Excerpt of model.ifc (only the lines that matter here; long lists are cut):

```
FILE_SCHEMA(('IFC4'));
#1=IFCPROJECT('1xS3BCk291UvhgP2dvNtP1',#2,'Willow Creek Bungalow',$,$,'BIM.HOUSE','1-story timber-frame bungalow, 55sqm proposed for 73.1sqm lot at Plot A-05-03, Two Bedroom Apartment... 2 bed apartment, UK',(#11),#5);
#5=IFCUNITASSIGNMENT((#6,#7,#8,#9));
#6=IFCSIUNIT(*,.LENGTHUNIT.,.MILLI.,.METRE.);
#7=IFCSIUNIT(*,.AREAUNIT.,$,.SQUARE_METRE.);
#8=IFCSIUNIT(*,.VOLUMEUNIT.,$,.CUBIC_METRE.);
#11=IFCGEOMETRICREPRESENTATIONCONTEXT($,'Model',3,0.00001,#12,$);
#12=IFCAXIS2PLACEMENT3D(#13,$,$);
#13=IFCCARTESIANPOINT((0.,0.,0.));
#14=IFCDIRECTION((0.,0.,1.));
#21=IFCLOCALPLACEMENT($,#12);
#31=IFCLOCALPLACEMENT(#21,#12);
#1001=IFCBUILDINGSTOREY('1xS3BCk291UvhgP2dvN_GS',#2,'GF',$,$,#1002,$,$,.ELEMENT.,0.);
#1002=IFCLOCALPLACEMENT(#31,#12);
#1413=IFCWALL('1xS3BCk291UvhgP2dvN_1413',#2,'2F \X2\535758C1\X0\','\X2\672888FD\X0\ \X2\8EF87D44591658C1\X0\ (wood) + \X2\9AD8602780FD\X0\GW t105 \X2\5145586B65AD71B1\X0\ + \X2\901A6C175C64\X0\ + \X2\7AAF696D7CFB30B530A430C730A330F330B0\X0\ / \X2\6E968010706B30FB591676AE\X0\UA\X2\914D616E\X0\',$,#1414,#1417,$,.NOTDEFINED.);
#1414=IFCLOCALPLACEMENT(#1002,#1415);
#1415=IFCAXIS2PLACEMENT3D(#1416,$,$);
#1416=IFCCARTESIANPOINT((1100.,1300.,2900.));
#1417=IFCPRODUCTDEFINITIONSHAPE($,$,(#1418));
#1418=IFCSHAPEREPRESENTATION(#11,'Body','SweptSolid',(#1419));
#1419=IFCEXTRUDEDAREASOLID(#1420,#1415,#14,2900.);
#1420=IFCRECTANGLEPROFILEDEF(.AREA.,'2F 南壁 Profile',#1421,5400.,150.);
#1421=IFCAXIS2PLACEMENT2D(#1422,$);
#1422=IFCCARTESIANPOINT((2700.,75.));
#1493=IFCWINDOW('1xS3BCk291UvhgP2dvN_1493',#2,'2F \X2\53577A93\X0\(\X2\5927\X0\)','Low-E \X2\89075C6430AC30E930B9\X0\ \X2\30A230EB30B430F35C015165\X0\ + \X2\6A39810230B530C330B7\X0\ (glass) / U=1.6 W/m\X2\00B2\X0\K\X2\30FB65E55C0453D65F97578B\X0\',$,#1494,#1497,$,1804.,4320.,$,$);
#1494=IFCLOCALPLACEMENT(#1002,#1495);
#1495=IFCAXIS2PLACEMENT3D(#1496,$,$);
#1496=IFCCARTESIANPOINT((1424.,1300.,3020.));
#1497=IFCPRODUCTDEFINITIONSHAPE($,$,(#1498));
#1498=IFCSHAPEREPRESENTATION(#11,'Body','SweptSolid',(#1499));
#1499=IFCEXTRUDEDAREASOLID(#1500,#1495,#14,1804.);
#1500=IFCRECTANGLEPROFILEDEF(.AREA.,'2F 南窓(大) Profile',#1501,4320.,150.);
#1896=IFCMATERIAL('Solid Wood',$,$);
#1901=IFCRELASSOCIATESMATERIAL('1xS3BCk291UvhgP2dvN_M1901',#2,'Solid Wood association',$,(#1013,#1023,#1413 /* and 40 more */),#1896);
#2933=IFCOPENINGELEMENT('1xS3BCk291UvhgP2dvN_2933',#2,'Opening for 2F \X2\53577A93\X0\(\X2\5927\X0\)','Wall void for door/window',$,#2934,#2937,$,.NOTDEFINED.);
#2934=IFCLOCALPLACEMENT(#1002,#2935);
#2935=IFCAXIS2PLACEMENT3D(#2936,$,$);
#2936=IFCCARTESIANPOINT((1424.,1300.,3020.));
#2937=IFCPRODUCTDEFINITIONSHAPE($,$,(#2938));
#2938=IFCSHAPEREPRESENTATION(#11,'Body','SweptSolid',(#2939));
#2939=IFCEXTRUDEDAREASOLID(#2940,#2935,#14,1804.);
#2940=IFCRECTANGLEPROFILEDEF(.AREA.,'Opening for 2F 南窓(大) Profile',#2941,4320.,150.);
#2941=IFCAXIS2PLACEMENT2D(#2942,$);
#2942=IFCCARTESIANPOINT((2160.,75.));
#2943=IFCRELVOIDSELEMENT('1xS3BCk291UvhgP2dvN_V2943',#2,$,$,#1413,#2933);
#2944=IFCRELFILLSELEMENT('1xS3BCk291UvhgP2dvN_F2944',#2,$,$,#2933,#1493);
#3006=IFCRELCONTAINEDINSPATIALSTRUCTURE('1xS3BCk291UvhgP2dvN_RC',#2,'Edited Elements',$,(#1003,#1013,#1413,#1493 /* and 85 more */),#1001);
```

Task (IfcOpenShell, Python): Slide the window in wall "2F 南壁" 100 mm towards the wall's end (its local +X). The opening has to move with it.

```python
import ifcopenshell
import ifcopenshell.api.geometry
import ifcopenshell.util.placement
import ifcopenshell.util.unit

model = ifcopenshell.open("model.ifc")
unit_scale = ifcopenshell.util.unit.calculate_unit_scale(model)

window = model.by_guid("1xS3BCk291UvhgP2dvN_1493")
opening = window.FillsVoids[0].RelatingOpeningElement
wall = opening.VoidsElements[0].RelatingBuildingElement

wall_matrix = ifcopenshell.util.placement.get_local_placement(wall.ObjectPlacement)
shift = wall_matrix[:3, 0] * 0.1 / unit_scale
before = ifcopenshell.util.placement.get_local_placement(window.ObjectPlacement)[:3, 3].copy()

# The window is not placed relative to its opening, so move both.
for product in (opening, window):
    matrix = ifcopenshell.util.placement.get_local_placement(product.ObjectPlacement)
    matrix[:3, 3] += shift
    ifcopenshell.api.geometry.edit_object_placement(model, product=product, matrix=matrix, is_si=False)

after = ifcopenshell.util.placement.get_local_placement(window.ObjectPlacement)[:3, 3]
print("window moved by", (after - before).round(3) + 0.0)

model.write("model_updated.ifc")
```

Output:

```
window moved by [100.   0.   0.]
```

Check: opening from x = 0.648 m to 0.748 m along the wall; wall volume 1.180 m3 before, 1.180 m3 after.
